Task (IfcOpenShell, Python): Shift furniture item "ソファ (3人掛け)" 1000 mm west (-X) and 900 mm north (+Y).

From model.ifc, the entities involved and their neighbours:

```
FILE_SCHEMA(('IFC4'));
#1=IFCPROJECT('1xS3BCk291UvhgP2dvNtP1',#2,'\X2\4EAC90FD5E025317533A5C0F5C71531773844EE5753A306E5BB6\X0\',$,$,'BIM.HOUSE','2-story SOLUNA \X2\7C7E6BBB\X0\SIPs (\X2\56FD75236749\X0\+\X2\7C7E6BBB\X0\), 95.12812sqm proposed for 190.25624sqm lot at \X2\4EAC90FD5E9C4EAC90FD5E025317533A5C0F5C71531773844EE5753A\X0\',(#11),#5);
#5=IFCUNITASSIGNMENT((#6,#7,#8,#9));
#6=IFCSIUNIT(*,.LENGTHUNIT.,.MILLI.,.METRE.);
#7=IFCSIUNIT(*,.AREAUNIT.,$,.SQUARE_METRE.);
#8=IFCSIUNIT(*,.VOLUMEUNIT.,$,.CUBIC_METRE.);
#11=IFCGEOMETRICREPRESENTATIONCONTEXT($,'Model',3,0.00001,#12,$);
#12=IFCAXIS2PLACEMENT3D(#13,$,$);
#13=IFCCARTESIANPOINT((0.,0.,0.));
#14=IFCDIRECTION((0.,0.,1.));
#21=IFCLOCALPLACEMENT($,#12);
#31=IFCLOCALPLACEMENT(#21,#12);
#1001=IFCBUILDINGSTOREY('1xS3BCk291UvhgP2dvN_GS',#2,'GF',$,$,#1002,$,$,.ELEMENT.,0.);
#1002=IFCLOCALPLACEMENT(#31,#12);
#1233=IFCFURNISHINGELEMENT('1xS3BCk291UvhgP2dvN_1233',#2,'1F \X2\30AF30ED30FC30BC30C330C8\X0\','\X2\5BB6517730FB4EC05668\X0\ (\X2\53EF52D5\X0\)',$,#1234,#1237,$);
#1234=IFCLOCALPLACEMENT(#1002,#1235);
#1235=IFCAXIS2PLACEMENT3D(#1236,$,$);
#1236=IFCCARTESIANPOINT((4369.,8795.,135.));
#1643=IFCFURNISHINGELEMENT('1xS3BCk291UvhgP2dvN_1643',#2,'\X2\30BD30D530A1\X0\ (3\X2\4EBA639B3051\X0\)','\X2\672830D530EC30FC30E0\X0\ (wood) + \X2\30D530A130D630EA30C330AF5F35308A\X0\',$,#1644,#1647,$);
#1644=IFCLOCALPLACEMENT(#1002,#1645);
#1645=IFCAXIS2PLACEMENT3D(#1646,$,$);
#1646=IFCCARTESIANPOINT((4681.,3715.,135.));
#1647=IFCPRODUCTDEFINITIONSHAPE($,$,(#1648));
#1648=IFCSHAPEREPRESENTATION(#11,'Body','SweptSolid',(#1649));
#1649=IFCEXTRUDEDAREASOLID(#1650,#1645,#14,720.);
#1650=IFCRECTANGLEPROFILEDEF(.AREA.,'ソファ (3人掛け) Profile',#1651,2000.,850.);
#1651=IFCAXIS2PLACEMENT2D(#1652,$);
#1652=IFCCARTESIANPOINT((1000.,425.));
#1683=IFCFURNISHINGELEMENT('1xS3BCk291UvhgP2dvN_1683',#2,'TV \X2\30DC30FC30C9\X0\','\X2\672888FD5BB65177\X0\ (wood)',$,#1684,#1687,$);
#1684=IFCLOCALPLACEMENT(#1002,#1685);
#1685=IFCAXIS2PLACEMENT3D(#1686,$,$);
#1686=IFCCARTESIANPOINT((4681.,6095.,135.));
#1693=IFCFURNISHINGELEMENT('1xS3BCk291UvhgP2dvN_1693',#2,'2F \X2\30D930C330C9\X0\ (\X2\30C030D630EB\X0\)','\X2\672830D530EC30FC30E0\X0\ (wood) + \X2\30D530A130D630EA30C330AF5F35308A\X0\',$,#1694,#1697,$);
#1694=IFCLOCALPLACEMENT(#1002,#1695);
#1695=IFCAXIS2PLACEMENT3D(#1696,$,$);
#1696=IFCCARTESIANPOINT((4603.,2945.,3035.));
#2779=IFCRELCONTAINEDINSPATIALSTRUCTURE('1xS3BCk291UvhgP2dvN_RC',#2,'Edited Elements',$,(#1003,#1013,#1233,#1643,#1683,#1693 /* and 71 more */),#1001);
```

```python
import ifcopenshell
import ifcopenshell.api.geometry
import ifcopenshell.util.placement
import ifcopenshell.util.unit

model = ifcopenshell.open("model.ifc")
unit_scale = ifcopenshell.util.unit.calculate_unit_scale(model)

item = model.by_guid("1xS3BCk291UvhgP2dvN_1643")
matrix = ifcopenshell.util.placement.get_local_placement(item.ObjectPlacement)
matrix[0, 3] -= 1 / unit_scale
matrix[1, 3] += 0.9 / unit_scale
ifcopenshell.api.geometry.edit_object_placement(model, product=item, matrix=matrix, is_si=False)

print(ifcopenshell.util.placement.get_local_placement(item.ObjectPlacement).round(3) + 0.0)

model.write("model-out.ifc")
```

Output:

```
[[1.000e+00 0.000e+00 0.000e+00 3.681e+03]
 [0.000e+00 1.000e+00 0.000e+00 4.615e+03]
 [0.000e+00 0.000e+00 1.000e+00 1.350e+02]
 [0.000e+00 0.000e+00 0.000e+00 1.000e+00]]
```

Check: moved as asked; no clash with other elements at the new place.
